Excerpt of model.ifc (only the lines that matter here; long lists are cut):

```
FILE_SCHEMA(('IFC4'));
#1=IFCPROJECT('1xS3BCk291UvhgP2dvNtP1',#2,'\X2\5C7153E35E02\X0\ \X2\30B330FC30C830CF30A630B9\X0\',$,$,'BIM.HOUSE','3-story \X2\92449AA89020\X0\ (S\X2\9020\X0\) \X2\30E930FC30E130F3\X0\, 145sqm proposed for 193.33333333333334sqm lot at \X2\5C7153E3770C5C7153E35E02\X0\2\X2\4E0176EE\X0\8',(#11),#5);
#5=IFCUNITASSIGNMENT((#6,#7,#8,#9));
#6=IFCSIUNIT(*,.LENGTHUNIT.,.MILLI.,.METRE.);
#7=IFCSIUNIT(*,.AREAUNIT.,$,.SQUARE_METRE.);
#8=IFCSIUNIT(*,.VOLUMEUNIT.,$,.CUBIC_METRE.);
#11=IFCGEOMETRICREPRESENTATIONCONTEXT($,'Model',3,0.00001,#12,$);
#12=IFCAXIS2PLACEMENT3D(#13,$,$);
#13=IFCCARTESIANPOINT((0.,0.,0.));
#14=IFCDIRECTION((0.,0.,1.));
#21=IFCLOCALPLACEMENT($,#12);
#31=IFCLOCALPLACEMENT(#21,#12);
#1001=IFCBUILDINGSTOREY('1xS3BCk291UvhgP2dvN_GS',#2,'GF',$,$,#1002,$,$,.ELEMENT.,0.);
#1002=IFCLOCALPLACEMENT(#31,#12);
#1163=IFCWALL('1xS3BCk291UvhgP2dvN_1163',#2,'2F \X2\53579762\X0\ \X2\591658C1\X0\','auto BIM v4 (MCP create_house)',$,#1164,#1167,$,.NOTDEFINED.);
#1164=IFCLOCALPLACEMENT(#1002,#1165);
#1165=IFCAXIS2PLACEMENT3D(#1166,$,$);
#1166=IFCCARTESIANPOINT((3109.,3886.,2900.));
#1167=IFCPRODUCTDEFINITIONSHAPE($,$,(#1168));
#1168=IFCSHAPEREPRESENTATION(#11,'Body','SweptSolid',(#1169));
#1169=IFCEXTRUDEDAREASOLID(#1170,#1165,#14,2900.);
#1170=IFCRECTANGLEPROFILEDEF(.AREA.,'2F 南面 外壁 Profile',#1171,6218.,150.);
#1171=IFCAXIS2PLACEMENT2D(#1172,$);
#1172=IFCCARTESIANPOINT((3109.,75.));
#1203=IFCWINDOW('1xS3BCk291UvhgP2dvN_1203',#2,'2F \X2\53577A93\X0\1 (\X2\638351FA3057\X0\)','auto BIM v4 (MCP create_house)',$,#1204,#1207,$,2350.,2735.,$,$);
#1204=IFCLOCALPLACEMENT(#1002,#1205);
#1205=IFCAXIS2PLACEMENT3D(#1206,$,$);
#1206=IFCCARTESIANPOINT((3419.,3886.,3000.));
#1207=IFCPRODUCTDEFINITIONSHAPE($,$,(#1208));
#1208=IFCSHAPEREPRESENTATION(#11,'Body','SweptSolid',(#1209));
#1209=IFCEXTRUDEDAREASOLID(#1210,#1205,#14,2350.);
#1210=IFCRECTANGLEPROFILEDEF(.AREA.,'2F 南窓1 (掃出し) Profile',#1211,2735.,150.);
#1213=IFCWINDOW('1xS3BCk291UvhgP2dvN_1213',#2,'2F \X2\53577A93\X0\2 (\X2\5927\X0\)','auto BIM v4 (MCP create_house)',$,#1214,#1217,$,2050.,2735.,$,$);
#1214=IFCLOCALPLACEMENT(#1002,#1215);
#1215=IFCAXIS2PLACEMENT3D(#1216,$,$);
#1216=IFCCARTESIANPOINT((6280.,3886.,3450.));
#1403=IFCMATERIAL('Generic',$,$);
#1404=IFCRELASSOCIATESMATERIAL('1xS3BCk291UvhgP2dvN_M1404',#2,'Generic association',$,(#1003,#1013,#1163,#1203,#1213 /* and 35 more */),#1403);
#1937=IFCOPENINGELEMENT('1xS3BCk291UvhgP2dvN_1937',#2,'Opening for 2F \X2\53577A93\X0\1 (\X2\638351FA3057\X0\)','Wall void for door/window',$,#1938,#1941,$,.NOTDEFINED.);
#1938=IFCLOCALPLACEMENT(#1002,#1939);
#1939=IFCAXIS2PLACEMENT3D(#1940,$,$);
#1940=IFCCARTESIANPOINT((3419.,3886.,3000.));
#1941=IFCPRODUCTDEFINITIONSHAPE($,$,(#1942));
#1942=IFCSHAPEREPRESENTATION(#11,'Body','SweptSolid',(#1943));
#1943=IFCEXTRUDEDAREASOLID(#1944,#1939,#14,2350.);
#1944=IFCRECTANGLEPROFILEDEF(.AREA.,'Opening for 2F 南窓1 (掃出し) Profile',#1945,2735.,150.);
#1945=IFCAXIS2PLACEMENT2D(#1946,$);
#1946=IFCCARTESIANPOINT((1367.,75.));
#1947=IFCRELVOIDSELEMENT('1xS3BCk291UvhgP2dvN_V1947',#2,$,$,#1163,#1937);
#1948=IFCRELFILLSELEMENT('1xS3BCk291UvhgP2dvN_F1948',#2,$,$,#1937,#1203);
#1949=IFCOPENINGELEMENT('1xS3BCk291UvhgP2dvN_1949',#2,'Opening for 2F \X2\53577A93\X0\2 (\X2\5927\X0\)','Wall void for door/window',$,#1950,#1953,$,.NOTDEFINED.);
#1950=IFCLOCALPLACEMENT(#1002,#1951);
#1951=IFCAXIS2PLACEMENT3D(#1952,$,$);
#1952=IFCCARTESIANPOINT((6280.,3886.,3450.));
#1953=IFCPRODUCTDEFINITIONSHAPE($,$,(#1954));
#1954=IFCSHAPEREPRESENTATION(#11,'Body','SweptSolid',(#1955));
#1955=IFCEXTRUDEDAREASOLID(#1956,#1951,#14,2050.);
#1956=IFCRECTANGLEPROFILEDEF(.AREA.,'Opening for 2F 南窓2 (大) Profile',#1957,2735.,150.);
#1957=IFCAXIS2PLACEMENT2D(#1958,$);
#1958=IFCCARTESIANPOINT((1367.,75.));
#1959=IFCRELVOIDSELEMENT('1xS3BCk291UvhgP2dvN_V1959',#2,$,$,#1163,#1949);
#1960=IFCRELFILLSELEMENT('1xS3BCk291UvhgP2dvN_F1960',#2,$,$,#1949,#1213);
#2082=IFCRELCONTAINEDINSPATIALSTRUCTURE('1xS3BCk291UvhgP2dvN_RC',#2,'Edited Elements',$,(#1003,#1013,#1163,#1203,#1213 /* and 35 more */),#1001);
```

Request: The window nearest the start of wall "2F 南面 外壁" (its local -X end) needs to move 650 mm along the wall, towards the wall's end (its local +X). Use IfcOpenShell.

```python
import ifcopenshell
import ifcopenshell.api.geometry
import ifcopenshell.util.placement

model = ifcopenshell.open("model.ifc")

window = model.by_guid("1xS3BCk291UvhgP2dvN_1203")
opening = window.FillsVoids[0].RelatingOpeningElement
wall = opening.VoidsElements[0].RelatingBuildingElement

wall_matrix = ifcopenshell.util.placement.get_local_placement(wall.ObjectPlacement)
shift = wall_matrix[:3, 0] * 650.0
before = ifcopenshell.util.placement.get_local_placement(window.ObjectPlacement)[:3, 3].copy()

# The window is not placed relative to its opening, so move both.
for product in (opening, window):
    matrix = ifcopenshell.util.placement.get_local_placement(product.ObjectPlacement)
    matrix[:3, 3] += shift
    ifcopenshell.api.geometry.edit_object_placement(model, product=product, matrix=matrix, is_si=False)

after = ifcopenshell.util.placement.get_local_placement(window.ObjectPlacement)[:3, 3]
print("window moved by", (after - before).round(3) + 0.0)

model.write("model_rev.ifc")
```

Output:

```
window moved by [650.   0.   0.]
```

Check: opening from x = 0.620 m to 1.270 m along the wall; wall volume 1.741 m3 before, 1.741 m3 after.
